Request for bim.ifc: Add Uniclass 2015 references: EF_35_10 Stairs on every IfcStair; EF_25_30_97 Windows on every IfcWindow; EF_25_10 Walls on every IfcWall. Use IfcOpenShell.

First a look at what the model holds.

```python
import ifcopenshell

model = ifcopenshell.open("bim.ifc")
print(model.schema)
print("classifications:", [c.Name for c in model.by_type("IfcClassification")])
for ifc_class in ("IfcDoor", "IfcRoof", "IfcStair", "IfcWall", "IfcWindow"):
    print(ifc_class, len(model.by_type(ifc_class)))
```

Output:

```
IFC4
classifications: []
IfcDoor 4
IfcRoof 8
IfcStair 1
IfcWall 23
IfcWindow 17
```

```python
import ifcopenshell
import ifcopenshell.api.classification

model = ifcopenshell.open("bim.ifc")

system = ifcopenshell.api.classification.add_classification(model, classification="Uniclass 2015")

codes = {
    "IfcStair": ("EF_35_10", "Stairs"),
    "IfcWindow": ("EF_25_30_97", "Windows"),
    "IfcWall": ("EF_25_10", "Walls"),
}
for ifc_class, (code, name) in codes.items():
    products = model.by_type(ifc_class)
    ifcopenshell.api.classification.add_reference(
        model, products=products, classification=system, identification=code, name=name
    )
    print(code, len(products))

model.write("bim-out.ifc")
```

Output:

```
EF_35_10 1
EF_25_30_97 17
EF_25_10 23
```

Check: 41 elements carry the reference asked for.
